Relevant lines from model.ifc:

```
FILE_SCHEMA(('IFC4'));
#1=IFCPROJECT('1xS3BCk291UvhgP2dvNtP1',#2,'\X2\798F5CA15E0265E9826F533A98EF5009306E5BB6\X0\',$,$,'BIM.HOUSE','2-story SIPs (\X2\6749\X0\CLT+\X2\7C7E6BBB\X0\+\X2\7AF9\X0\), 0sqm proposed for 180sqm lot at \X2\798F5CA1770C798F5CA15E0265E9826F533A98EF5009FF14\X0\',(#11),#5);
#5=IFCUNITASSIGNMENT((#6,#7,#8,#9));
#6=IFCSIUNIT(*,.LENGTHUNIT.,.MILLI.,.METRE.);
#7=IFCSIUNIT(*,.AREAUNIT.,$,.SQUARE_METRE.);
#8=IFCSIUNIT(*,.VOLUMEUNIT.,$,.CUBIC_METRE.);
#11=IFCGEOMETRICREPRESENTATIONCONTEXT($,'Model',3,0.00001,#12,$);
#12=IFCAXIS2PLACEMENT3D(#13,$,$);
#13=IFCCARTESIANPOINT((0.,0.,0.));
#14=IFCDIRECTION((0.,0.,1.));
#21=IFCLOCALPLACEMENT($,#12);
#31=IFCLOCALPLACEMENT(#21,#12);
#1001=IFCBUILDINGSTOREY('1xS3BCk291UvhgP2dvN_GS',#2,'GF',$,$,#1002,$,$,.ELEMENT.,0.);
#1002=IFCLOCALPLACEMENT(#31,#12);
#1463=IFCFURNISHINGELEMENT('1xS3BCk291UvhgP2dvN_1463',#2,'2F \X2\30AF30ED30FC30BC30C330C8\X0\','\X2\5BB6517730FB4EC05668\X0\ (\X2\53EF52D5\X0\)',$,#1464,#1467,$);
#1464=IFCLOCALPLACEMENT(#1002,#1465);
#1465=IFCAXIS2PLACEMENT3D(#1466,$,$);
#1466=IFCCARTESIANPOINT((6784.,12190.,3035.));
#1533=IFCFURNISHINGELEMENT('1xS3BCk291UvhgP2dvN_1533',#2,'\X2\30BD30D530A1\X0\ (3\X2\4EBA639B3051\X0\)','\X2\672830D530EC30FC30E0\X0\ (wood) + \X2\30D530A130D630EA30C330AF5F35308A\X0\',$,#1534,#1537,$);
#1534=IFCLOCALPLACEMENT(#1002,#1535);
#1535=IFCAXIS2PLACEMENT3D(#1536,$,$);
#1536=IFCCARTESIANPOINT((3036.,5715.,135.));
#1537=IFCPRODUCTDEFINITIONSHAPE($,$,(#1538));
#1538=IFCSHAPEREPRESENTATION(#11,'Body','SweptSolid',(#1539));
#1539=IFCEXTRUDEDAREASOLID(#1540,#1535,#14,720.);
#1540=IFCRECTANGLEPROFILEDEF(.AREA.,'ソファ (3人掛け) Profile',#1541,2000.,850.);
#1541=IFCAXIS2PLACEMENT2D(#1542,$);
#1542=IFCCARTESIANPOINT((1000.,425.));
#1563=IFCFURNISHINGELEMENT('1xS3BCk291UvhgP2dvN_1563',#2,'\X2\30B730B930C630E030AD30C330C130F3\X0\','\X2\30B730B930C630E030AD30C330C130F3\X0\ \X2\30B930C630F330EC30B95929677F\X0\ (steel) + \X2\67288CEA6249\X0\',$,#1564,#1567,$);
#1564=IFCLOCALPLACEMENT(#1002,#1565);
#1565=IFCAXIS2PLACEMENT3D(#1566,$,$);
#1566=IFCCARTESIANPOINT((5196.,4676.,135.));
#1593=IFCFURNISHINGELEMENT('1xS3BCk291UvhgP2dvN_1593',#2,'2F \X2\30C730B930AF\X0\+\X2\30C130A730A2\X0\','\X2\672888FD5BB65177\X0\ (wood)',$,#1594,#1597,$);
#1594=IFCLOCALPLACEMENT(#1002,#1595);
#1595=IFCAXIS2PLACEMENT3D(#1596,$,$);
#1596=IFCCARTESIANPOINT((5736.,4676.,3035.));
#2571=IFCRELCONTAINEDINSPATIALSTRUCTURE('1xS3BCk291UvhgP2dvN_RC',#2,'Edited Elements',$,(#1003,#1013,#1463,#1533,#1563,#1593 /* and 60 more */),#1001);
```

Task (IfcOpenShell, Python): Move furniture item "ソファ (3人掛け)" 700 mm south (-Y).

```python
import ifcopenshell
import ifcopenshell.api.geometry
import ifcopenshell.util.placement

model = ifcopenshell.open("model.ifc")

item = model.by_guid("1xS3BCk291UvhgP2dvN_1533")
matrix = ifcopenshell.util.placement.get_local_placement(item.ObjectPlacement)
matrix[1, 3] -= 700.0
ifcopenshell.api.geometry.edit_object_placement(model, product=item, matrix=matrix, is_si=False)

print(ifcopenshell.util.placement.get_local_placement(item.ObjectPlacement).round(3) + 0.0)

model.write("model_edited.ifc")
```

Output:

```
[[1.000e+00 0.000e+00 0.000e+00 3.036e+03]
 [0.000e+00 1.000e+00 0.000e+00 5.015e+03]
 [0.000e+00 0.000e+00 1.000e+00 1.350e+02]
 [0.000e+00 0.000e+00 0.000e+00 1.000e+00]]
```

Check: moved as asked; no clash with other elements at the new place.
